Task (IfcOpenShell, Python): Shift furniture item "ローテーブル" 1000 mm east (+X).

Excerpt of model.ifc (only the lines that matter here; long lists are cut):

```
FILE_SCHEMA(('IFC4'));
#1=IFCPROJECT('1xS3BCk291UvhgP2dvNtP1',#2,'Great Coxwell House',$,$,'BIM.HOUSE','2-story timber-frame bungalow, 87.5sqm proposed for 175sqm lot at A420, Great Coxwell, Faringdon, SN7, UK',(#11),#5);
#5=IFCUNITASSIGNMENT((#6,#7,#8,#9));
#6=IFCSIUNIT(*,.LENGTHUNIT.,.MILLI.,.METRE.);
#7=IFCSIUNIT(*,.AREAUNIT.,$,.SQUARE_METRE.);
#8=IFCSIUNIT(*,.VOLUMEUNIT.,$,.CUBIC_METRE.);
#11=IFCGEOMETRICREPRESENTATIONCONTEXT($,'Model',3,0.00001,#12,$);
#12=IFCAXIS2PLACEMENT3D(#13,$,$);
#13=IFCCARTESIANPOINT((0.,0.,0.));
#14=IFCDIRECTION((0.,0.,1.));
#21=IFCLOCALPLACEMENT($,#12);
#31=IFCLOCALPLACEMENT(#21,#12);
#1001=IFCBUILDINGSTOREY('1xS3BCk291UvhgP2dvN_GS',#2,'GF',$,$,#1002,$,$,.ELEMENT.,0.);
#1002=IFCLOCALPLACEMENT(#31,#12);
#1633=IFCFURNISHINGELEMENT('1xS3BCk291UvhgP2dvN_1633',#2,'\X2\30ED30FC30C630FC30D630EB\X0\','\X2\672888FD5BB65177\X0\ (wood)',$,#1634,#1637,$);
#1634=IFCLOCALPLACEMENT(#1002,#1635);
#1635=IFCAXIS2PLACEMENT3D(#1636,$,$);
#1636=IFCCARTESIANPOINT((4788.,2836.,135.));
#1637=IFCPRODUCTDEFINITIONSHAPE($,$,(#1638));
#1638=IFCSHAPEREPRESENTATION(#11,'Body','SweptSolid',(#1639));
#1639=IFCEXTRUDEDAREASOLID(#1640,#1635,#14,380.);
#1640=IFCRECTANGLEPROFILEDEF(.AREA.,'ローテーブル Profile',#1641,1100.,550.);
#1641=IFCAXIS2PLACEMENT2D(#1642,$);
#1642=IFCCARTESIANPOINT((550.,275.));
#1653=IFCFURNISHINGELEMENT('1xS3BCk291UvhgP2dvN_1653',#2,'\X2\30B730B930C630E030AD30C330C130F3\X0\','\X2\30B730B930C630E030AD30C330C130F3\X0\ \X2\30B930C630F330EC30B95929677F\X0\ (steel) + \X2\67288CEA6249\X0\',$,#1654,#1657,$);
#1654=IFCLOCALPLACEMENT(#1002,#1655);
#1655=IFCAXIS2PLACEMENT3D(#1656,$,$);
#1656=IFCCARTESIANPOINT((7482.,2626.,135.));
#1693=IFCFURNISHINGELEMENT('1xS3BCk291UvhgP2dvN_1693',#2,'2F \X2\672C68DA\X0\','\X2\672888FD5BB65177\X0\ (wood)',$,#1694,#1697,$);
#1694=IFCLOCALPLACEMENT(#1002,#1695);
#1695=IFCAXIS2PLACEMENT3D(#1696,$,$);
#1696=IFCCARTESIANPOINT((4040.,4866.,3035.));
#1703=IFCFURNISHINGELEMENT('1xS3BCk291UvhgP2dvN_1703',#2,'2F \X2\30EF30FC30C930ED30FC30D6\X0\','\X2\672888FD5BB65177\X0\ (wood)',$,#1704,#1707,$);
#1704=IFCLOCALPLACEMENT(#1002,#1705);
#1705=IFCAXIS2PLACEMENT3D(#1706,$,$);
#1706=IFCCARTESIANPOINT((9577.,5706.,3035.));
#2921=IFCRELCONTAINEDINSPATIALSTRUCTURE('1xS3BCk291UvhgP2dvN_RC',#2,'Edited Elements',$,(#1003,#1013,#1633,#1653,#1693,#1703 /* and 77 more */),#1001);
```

```python
import ifcopenshell
import ifcopenshell.api.geometry
import ifcopenshell.util.placement
import ifcopenshell.util.unit

model = ifcopenshell.open("model.ifc")
unit_scale = ifcopenshell.util.unit.calculate_unit_scale(model)

item = model.by_guid("1xS3BCk291UvhgP2dvN_1633")
matrix = ifcopenshell.util.placement.get_local_placement(item.ObjectPlacement)
matrix[0, 3] += 1 / unit_scale
ifcopenshell.api.geometry.edit_object_placement(model, product=item, matrix=matrix, is_si=False)

print(ifcopenshell.util.placement.get_local_placement(item.ObjectPlacement).round(3) + 0.0)

model.write("model_updated.ifc")
```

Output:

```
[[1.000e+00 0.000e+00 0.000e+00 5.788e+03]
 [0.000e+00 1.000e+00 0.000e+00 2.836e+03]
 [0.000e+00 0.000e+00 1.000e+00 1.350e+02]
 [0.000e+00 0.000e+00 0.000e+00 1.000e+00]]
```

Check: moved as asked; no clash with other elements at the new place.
